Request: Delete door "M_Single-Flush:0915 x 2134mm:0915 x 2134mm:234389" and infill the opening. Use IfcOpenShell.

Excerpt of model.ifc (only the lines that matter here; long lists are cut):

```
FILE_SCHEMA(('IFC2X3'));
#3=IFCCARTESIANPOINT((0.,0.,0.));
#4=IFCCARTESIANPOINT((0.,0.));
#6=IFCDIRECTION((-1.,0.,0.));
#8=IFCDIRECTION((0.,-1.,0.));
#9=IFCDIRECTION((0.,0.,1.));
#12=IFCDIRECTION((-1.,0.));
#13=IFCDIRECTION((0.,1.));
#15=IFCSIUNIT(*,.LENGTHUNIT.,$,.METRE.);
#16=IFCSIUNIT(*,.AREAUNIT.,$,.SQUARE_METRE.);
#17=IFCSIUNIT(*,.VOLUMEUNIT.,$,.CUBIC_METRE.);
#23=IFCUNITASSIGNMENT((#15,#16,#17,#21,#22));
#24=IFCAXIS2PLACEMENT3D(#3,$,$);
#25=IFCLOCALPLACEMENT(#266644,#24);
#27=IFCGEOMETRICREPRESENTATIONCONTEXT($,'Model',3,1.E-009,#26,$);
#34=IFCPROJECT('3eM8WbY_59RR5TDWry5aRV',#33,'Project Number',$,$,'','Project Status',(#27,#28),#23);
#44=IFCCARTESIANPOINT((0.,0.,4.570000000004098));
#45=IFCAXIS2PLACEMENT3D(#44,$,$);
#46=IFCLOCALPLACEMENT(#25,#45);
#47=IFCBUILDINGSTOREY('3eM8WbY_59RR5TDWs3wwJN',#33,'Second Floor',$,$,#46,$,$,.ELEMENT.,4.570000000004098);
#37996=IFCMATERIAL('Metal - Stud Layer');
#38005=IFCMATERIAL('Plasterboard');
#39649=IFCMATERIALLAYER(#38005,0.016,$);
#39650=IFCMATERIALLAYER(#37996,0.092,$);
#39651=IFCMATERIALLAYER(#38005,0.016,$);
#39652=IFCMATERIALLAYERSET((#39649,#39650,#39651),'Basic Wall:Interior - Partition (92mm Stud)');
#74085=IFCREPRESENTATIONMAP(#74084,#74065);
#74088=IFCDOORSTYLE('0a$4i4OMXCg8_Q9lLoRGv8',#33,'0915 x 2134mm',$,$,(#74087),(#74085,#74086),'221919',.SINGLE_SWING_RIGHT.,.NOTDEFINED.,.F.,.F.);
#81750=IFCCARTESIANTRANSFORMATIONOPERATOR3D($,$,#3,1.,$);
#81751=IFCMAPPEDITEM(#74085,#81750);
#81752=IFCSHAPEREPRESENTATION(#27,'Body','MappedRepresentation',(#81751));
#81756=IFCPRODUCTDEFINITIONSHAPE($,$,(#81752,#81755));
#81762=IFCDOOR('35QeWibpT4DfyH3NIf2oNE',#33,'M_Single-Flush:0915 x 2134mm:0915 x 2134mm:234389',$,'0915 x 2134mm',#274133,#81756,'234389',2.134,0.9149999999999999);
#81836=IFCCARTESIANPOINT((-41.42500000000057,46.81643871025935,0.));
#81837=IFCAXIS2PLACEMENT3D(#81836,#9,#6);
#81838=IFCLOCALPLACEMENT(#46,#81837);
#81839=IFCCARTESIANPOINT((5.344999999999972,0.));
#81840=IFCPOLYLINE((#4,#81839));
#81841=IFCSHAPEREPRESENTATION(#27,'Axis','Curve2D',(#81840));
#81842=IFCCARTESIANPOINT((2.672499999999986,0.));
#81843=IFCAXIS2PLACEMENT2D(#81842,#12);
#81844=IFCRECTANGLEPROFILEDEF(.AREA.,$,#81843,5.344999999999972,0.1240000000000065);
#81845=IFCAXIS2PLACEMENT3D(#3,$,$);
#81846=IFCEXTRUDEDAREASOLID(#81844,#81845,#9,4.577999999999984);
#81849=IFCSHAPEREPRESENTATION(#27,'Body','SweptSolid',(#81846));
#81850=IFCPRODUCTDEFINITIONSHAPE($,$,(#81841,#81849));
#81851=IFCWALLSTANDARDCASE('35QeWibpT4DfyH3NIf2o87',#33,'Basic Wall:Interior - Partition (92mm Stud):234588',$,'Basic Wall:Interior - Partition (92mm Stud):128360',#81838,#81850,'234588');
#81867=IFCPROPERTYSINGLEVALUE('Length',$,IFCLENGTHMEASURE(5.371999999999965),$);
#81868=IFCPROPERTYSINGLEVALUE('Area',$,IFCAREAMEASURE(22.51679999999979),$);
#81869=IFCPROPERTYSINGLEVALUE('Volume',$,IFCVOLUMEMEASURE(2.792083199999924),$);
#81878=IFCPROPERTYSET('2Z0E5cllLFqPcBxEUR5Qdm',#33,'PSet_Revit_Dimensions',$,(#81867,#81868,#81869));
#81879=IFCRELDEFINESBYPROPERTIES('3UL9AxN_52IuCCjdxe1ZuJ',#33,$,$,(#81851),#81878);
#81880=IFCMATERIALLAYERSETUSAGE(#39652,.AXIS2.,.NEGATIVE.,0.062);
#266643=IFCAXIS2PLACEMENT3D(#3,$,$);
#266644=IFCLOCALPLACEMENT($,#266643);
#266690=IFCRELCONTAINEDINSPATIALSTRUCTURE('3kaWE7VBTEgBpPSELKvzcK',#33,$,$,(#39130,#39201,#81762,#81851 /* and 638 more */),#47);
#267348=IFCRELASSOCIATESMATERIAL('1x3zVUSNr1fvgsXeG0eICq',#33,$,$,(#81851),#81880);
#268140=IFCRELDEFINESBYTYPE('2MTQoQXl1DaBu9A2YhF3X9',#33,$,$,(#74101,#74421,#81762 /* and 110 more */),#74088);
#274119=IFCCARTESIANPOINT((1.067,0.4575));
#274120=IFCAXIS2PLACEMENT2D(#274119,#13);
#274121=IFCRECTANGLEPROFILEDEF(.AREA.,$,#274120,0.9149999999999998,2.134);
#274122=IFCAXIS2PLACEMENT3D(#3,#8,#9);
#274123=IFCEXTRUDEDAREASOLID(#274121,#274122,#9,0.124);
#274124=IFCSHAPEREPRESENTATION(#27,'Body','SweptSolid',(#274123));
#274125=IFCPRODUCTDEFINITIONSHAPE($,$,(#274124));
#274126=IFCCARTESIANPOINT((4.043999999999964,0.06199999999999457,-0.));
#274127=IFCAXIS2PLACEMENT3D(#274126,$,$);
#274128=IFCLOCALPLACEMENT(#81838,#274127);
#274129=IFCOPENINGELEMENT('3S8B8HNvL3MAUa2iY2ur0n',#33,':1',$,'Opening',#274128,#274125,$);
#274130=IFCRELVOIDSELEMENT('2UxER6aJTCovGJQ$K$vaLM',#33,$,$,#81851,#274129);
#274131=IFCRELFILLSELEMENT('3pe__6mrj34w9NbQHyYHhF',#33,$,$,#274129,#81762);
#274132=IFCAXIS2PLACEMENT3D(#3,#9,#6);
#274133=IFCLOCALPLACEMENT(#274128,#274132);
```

```python
import ifcopenshell
import ifcopenshell.api.feature
import ifcopenshell.api.pset
import ifcopenshell.api.root
import ifcopenshell.geom
import ifcopenshell.util.element
import ifcopenshell.util.shape
import ifcopenshell.util.unit

model = ifcopenshell.open("model.ifc")
area_scale = ifcopenshell.util.unit.calculate_unit_scale(model, "AREAUNIT")
volume_scale = ifcopenshell.util.unit.calculate_unit_scale(model, "VOLUMEUNIT")
settings = ifcopenshell.geom.settings()


def volume(element):
    """Net volume in cubic metres, openings subtracted."""
    shape = ifcopenshell.geom.create_shape(settings, element)
    return ifcopenshell.util.shape.get_volume(shape.geometry)


door = model.by_guid("35QeWibpT4DfyH3NIf2oNE")
opening = door.FillsVoids[0].RelatingOpeningElement
wall = opening.VoidsElements[0].RelatingBuildingElement
before = volume(wall)

ifcopenshell.api.root.remove_product(model, product=door)
ifcopenshell.api.feature.remove_feature(model, feature=opening)

after = volume(wall)
thickness = 0.124  # wall thickness in metres

# Update the wall's stored quantities.
pset = model.by_id(ifcopenshell.util.element.get_pset(wall, "PSet_Revit_Dimensions", should_inherit=False)["id"])
ifcopenshell.api.pset.edit_pset(model, pset=pset, properties={
    "Area": model.create_entity("IfcAreaMeasure", after / thickness / area_scale),
    "Volume": model.create_entity("IfcVolumeMeasure", after / volume_scale),
})

print(f"wall volume {before:.3f} -> {after:.3f} m3")

model.write("model_v2.ifc")
```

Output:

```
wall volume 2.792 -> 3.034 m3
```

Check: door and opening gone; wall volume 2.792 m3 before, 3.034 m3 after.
